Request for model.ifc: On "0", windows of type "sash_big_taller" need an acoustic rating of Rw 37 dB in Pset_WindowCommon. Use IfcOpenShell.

First a look at what the model holds.

```python
import ifcopenshell
import ifcopenshell.util.element

model = ifcopenshell.open("model.ifc")
print(model.schema)
storey = next(s for s in model.by_type("IfcBuildingStorey") if s.Name == "0")
windows = [e for e in ifcopenshell.util.element.get_decomposition(storey) if e.is_a("IfcWindow")]
seen = {}
for e in windows:
    element_type = ifcopenshell.util.element.get_type(e)
    key = (element_type.Name if element_type != e and element_type else None, ifcopenshell.util.element.get_pset(e, "Pset_WindowCommon", "AcousticRating"))
    seen[key] = seen.get(key, 0) + 1
for (name, value), count in sorted(seen.items(), key=str):
    print(count, "x", name, "|", value)
```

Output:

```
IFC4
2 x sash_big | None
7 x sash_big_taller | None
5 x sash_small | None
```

```python
import ifcopenshell
import ifcopenshell.api.pset
import ifcopenshell.util.element

model = ifcopenshell.open("model.ifc")

storey = next(s for s in model.by_type("IfcBuildingStorey") if s.Name == "0")
windows = [e for e in ifcopenshell.util.element.get_decomposition(storey) if e.is_a("IfcWindow")]

count = 0
for e in windows:
    element_type = ifcopenshell.util.element.get_type(e)
    if element_type in (None, e) or element_type.Name != "sash_big_taller":
        continue
    # add_pset returns the element's existing set when there is one.
    pset = ifcopenshell.api.pset.add_pset(model, product=e, name="Pset_WindowCommon")
    ifcopenshell.api.pset.edit_pset(model, pset=pset, properties={"AcousticRating": "Rw 37 dB"})
    count += 1

print(count, "windows updated")

model.write("model_v2.ifc")
```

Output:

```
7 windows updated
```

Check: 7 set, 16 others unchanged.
